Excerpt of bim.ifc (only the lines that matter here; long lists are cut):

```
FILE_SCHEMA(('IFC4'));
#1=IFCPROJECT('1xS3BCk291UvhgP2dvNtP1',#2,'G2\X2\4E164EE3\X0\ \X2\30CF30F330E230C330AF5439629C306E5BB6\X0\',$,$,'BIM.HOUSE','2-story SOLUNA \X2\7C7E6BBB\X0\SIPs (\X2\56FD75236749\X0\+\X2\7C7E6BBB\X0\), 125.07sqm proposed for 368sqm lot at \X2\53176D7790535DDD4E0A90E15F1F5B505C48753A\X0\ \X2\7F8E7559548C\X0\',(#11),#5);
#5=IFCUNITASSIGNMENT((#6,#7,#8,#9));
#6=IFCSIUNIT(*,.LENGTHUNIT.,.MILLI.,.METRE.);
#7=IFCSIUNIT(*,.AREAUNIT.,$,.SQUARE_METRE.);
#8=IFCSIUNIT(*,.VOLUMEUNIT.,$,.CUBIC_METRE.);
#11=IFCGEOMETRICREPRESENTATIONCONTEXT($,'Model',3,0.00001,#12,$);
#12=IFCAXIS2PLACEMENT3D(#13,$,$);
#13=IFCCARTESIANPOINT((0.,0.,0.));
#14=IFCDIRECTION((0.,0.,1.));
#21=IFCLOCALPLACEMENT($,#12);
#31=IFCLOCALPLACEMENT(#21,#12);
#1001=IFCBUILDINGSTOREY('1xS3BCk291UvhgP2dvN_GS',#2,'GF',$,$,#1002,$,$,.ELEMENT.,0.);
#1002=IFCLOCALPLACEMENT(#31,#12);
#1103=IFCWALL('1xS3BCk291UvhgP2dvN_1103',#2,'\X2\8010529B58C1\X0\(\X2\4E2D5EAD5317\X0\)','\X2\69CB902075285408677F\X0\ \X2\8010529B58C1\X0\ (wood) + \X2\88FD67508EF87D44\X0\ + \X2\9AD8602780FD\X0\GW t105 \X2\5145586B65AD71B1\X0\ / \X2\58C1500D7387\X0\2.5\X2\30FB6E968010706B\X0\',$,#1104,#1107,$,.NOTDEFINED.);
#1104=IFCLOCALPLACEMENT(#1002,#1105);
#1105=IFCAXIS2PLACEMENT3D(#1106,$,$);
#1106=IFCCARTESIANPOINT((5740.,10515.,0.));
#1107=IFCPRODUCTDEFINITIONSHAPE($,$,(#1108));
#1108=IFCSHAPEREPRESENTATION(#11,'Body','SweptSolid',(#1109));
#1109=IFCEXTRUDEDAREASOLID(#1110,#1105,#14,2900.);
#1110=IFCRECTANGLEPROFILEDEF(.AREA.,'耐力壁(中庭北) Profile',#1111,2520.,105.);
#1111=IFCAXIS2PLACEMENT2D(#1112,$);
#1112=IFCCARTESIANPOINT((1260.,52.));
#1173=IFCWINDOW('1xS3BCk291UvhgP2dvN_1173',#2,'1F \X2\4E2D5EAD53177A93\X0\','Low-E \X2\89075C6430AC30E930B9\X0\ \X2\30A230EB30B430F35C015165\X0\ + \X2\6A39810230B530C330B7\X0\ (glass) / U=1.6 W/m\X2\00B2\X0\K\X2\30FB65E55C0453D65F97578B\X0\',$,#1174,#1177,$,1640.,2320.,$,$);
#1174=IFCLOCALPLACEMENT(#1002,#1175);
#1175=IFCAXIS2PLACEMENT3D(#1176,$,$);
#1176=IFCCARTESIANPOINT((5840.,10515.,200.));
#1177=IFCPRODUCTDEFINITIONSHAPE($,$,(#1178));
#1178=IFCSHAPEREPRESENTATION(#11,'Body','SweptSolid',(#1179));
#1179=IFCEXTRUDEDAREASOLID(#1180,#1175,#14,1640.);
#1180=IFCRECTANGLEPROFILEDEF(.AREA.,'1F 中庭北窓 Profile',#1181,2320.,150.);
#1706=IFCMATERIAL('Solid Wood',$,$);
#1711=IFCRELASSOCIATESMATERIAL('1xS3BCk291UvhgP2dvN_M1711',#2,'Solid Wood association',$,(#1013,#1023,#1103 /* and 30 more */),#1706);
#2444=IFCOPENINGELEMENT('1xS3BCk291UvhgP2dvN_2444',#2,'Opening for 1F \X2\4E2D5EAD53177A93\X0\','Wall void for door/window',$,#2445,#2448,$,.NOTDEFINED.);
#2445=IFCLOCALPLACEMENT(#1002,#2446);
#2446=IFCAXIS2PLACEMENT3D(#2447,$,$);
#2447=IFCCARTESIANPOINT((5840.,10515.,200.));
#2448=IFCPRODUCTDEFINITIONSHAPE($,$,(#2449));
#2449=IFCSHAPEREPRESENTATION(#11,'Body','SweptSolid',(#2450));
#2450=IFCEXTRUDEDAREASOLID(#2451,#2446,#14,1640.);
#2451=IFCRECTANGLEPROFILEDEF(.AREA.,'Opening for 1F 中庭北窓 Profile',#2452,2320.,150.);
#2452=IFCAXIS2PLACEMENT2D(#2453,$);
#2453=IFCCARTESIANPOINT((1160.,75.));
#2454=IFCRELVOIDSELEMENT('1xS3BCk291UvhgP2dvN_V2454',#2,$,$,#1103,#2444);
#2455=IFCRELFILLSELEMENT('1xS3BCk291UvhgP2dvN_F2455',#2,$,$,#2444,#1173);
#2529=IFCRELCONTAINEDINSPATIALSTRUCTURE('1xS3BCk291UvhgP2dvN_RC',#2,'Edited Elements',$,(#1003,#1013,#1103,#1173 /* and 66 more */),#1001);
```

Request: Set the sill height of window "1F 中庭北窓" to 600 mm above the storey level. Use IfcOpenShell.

```python
import numpy as np
import ifcopenshell
import ifcopenshell.api.geometry
import ifcopenshell.geom
import ifcopenshell.util.element
import ifcopenshell.util.placement
import ifcopenshell.util.shape
import ifcopenshell.util.unit

model = ifcopenshell.open("bim.ifc")
unit_scale = ifcopenshell.util.unit.calculate_unit_scale(model)

window = model.by_guid("1xS3BCk291UvhgP2dvN_1173")
opening = window.FillsVoids[0].RelatingOpeningElement
storey = ifcopenshell.util.element.get_container(window, ifc_class="IfcBuildingStorey")
level = ifcopenshell.util.placement.get_local_placement(storey.ObjectPlacement)[2, 3]

# The opening's origin need not be at the sill, so measure its lowest point.
shape = ifcopenshell.geom.create_shape(ifcopenshell.geom.settings(), opening)
bottom = ifcopenshell.util.shape.get_shape_bottom_elevation(shape, shape.geometry) / unit_scale
dz = level + 0.6 / unit_scale - bottom

shift = np.array([0.0, 0.0, dz])
# The window is not placed relative to its opening, so move both.
for product in (opening, window):
    matrix = ifcopenshell.util.placement.get_local_placement(product.ObjectPlacement)
    matrix[:3, 3] += shift
    ifcopenshell.api.geometry.edit_object_placement(model, product=product, matrix=matrix, is_si=False)

print(f"moved by {dz * unit_scale:+.3f} m")

model.write("bim-out.ifc")
```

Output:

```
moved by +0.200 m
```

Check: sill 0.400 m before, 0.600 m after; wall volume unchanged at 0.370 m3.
